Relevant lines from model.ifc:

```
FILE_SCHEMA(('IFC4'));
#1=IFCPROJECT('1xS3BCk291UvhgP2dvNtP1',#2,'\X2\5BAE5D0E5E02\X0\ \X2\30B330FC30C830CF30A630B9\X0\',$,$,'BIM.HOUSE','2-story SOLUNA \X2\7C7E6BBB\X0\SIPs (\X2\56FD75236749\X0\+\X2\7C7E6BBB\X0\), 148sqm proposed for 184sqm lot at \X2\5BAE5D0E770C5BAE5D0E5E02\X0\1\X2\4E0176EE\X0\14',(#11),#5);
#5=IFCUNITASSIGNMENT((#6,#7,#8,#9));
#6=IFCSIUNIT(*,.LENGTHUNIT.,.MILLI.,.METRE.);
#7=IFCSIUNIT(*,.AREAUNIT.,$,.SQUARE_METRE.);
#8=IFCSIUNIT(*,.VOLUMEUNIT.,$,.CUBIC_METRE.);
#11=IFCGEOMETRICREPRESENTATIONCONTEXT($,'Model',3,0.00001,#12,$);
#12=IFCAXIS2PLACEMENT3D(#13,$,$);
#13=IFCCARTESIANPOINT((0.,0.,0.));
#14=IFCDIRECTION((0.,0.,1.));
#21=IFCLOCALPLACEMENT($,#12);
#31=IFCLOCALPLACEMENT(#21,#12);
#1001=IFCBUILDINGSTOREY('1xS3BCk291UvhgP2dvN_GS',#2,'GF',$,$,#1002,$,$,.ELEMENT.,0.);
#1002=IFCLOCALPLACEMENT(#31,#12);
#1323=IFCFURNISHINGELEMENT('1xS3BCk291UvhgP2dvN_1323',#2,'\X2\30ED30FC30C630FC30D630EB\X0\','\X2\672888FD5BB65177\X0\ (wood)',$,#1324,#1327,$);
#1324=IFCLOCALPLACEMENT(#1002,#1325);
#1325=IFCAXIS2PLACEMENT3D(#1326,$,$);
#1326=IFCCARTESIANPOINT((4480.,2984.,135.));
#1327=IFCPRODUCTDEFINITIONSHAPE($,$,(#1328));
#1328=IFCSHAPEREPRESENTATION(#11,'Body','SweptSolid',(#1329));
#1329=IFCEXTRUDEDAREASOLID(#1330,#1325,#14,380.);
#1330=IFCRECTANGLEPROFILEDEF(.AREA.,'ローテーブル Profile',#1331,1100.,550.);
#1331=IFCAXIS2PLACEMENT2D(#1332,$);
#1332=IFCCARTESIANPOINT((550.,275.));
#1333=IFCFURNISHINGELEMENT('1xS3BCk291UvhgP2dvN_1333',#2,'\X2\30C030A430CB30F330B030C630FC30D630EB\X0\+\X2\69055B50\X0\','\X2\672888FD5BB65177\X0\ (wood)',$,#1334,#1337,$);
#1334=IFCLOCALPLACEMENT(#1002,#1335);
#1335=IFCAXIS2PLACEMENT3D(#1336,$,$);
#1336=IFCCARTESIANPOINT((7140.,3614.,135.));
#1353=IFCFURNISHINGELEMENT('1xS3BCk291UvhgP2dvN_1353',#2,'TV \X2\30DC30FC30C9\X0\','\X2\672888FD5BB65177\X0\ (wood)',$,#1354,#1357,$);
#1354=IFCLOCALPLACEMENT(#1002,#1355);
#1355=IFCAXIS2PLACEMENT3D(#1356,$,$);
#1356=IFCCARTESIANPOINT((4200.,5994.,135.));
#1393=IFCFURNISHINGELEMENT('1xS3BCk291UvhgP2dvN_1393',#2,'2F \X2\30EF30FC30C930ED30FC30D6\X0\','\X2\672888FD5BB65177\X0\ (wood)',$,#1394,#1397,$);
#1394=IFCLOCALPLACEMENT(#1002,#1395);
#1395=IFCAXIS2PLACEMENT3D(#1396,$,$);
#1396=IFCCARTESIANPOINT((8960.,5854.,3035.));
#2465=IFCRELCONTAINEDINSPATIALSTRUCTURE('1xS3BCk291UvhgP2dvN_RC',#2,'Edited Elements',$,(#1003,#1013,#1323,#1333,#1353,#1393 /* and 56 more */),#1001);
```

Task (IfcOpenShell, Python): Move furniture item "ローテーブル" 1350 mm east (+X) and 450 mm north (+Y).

```python
import ifcopenshell
import ifcopenshell.api.geometry
import ifcopenshell.util.placement
import ifcopenshell.util.unit

model = ifcopenshell.open("model.ifc")
unit_scale = ifcopenshell.util.unit.calculate_unit_scale(model)

item = model.by_guid("1xS3BCk291UvhgP2dvN_1323")
matrix = ifcopenshell.util.placement.get_local_placement(item.ObjectPlacement)
matrix[0, 3] += 1.35 / unit_scale
matrix[1, 3] += 0.45 / unit_scale
ifcopenshell.api.geometry.edit_object_placement(model, product=item, matrix=matrix, is_si=False)

print(ifcopenshell.util.placement.get_local_placement(item.ObjectPlacement).round(3) + 0.0)

model.write("model-out.ifc")
```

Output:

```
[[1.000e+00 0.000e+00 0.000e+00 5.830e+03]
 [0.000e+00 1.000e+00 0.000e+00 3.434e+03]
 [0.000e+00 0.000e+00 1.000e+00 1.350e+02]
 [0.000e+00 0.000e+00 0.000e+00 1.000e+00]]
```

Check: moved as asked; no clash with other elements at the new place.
